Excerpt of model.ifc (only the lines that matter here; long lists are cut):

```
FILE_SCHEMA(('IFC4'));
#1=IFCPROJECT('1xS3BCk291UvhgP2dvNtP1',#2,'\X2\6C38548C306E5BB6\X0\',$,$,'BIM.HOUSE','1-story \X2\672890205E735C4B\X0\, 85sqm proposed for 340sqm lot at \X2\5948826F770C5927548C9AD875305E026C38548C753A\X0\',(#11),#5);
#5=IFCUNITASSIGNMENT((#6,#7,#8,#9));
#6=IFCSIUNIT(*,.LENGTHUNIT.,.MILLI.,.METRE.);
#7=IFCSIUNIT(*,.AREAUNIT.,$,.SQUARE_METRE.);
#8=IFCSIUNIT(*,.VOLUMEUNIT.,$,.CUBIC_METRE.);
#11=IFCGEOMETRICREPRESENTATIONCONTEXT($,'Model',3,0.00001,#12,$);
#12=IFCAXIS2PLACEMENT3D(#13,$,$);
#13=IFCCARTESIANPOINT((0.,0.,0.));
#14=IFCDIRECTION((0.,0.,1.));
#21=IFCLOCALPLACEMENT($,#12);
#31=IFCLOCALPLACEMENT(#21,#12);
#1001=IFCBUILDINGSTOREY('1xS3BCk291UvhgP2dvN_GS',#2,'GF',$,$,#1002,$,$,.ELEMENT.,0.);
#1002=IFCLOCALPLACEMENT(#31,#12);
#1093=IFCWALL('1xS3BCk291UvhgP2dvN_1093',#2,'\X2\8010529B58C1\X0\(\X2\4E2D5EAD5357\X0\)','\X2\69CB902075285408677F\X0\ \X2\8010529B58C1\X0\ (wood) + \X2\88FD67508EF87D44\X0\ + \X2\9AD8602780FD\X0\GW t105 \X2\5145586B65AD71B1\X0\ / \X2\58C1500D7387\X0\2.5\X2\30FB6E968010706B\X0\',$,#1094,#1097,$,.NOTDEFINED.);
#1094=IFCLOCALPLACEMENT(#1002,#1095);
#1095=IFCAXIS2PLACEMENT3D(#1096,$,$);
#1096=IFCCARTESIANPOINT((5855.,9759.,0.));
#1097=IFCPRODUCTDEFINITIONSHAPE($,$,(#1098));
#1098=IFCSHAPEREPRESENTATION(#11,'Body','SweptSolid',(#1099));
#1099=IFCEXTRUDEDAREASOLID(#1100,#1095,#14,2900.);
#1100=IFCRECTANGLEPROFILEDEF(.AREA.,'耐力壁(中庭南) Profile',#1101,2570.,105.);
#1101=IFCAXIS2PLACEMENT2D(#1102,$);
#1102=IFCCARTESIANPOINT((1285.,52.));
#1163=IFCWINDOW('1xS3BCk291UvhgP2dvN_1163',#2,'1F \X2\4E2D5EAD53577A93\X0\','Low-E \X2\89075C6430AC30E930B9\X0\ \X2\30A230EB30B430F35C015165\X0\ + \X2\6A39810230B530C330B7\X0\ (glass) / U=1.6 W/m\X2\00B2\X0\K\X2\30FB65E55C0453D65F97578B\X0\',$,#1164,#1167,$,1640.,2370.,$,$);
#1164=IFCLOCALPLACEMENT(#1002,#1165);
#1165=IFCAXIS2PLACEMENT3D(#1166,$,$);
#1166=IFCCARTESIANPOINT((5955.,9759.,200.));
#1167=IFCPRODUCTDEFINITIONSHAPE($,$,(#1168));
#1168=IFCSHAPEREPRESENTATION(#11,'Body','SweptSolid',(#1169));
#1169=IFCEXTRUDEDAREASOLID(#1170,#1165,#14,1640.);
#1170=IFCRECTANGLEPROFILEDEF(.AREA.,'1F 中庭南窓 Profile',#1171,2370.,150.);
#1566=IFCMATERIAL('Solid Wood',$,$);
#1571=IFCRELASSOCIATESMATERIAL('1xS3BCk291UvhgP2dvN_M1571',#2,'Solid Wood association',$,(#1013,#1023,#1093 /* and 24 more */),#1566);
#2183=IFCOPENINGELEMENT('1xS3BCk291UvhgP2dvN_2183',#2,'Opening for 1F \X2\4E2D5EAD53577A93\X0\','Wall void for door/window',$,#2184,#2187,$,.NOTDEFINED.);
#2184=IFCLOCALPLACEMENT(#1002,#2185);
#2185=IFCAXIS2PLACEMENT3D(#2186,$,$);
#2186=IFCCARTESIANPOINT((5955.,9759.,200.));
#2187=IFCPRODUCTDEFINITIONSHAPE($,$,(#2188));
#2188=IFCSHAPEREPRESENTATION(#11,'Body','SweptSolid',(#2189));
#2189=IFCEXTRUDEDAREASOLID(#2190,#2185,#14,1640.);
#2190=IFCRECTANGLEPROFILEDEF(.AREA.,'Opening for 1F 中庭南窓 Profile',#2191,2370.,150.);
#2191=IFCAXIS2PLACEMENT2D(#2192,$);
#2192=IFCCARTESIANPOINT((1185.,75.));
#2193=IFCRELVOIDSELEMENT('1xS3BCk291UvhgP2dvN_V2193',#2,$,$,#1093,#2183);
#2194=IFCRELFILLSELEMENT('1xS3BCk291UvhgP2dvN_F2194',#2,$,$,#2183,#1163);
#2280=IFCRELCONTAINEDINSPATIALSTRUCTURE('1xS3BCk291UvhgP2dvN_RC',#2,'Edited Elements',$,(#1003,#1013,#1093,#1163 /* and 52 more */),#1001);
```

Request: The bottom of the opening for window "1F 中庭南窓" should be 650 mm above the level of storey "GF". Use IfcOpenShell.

```python
import numpy as np
import ifcopenshell
import ifcopenshell.api.geometry
import ifcopenshell.geom
import ifcopenshell.util.element
import ifcopenshell.util.placement
import ifcopenshell.util.shape
import ifcopenshell.util.unit

model = ifcopenshell.open("model.ifc")
unit_scale = ifcopenshell.util.unit.calculate_unit_scale(model)

window = model.by_id(1163)
opening = window.FillsVoids[0].RelatingOpeningElement
storey = ifcopenshell.util.element.get_container(window, ifc_class="IfcBuildingStorey")
level = ifcopenshell.util.placement.get_local_placement(storey.ObjectPlacement)[2, 3]

# The opening's origin need not be at the sill, so measure its lowest point.
shape = ifcopenshell.geom.create_shape(ifcopenshell.geom.settings(), opening)
bottom = ifcopenshell.util.shape.get_shape_bottom_elevation(shape, shape.geometry) / unit_scale
dz = level + 650.0 - bottom

shift = np.array([0.0, 0.0, dz])
# The window is not placed relative to its opening, so move both.
for product in (opening, window):
    matrix = ifcopenshell.util.placement.get_local_placement(product.ObjectPlacement)
    matrix[:3, 3] += shift
    ifcopenshell.api.geometry.edit_object_placement(model, product=product, matrix=matrix, is_si=False)

print(f"moved by {dz * unit_scale:+.3f} m")

model.write("model_edited.ifc")
```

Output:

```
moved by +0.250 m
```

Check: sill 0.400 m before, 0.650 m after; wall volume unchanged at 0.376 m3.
